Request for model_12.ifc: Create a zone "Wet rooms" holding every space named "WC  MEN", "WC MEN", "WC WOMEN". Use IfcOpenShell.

First a look at what the model holds.

```python
import ifcopenshell

model = ifcopenshell.open("model_12.ifc")
print(model.schema)
seen = {}
for space in model.by_type("IfcSpace"):
    seen[space.LongName] = seen.get(space.LongName, 0) + 1
for name, count in sorted(seen.items(), key=str):
    print(count, "x", name)
print("zones:", [z.Name for z in model.by_type("IfcZone")][:20])
```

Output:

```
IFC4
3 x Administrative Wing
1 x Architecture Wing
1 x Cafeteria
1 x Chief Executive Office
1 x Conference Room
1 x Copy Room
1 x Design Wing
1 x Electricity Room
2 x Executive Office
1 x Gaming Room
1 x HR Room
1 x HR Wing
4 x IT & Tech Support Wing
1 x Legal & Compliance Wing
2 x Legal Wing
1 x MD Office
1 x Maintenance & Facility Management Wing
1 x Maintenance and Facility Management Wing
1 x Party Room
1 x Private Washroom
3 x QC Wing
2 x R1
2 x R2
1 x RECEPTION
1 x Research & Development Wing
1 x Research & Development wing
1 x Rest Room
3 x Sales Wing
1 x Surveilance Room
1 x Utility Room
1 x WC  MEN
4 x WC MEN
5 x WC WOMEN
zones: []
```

```python
import ifcopenshell
import ifcopenshell.api.group
import ifcopenshell.api.root

model = ifcopenshell.open("model_12.ifc")

names = {"WC  MEN", "WC MEN", "WC WOMEN"}
spaces = [s for s in model.by_type("IfcSpace") if s.LongName in names]

zone = ifcopenshell.api.root.create_entity(model, ifc_class="IfcZone", name="Wet rooms")
ifcopenshell.api.group.assign_group(model, products=spaces, group=zone)
print(len(spaces), "spaces in", zone.Name)

model.write("model_12_v2.ifc")
```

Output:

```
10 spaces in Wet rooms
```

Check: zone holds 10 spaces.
